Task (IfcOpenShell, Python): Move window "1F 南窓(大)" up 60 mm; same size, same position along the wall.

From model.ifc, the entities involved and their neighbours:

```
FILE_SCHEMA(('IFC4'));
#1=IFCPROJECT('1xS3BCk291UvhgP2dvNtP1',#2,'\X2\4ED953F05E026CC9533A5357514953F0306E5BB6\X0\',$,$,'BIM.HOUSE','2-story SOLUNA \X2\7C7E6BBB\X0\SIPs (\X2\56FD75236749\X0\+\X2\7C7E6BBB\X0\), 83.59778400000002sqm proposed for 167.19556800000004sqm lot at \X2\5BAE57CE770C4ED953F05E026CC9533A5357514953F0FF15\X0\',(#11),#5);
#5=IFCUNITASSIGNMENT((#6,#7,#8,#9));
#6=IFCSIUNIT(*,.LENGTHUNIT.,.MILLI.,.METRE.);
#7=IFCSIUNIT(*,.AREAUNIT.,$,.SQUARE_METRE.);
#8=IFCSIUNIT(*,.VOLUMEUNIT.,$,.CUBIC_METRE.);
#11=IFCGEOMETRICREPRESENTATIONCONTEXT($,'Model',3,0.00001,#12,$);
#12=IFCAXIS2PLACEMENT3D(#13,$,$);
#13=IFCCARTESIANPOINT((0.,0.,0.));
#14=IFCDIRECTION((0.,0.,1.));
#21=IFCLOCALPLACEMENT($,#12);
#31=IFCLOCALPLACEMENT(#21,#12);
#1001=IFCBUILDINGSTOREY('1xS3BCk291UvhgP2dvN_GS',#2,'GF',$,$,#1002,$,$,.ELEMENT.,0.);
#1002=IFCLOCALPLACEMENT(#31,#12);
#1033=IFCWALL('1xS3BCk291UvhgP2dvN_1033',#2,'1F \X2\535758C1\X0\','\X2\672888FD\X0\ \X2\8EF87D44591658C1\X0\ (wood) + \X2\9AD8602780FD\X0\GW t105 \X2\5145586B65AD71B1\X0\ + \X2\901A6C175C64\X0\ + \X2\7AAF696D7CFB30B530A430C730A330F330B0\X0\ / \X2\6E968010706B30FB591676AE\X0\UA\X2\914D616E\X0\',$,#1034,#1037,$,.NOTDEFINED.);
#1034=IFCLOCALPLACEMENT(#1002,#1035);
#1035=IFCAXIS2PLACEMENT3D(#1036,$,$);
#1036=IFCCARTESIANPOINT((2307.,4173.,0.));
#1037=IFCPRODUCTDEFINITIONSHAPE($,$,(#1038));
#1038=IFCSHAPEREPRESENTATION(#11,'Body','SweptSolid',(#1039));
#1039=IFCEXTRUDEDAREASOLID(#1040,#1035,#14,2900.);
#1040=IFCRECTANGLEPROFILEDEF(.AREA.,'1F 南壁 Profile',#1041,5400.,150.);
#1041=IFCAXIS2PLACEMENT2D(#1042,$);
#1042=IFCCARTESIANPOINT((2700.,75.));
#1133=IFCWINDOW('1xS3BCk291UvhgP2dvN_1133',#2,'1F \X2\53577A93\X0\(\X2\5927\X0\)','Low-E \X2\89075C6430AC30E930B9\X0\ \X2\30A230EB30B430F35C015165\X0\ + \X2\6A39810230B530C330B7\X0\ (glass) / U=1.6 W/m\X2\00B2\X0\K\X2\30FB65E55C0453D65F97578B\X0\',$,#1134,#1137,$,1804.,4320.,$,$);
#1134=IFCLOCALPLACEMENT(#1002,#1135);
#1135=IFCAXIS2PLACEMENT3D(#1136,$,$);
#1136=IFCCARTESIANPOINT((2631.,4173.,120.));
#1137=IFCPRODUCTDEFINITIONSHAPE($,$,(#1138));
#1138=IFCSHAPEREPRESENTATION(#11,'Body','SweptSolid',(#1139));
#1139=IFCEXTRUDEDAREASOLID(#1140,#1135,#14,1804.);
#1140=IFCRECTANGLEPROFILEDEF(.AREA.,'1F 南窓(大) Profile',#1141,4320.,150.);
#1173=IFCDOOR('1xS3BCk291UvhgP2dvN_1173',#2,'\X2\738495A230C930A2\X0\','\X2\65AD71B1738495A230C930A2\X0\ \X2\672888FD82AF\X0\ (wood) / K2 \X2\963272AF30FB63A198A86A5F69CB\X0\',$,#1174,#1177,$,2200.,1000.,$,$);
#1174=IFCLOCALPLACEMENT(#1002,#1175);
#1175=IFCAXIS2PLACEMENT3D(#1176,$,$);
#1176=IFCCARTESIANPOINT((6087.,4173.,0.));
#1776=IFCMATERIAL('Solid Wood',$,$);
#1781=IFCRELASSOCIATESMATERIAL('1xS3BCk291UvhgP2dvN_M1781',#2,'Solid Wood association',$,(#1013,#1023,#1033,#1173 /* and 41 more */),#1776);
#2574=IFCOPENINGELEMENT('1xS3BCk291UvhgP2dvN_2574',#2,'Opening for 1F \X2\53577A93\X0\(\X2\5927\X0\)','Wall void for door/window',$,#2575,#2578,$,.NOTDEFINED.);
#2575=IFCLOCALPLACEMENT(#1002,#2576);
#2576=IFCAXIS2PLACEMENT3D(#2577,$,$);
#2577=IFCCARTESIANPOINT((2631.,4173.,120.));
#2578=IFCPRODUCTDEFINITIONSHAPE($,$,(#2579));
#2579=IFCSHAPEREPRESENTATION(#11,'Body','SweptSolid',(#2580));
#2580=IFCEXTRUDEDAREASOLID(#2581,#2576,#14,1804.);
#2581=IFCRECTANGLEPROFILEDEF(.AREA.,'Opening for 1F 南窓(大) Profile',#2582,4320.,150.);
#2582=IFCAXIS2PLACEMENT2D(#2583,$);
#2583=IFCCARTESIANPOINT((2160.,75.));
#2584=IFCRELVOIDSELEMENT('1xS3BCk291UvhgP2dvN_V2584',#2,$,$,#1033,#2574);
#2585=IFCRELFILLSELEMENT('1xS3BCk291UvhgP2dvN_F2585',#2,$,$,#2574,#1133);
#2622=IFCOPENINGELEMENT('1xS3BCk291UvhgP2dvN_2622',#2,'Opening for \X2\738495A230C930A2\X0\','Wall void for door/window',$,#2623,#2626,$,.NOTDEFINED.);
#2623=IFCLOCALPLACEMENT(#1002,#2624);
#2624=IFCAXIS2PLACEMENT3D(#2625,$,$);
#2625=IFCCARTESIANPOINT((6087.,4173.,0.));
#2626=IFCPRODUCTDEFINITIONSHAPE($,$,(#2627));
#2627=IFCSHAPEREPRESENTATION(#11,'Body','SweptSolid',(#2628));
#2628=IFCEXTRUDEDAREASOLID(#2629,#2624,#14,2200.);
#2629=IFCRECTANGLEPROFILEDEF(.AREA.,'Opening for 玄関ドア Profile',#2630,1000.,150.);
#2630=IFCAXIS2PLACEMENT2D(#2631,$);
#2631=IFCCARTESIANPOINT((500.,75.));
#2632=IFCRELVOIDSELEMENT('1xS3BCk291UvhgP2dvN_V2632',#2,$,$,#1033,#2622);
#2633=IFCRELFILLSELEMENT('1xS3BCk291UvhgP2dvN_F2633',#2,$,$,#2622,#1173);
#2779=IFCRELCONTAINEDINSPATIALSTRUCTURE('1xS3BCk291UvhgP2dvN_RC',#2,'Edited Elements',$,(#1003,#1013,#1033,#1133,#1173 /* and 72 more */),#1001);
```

```python
import numpy as np
import ifcopenshell
import ifcopenshell.api.geometry
import ifcopenshell.util.placement
import ifcopenshell.util.unit

model = ifcopenshell.open("model.ifc")
unit_scale = ifcopenshell.util.unit.calculate_unit_scale(model)

window = model.by_id(1133)
opening = window.FillsVoids[0].RelatingOpeningElement
dz = 0.06 / unit_scale

shift = np.array([0.0, 0.0, dz])
# The window is not placed relative to its opening, so move both.
for product in (opening, window):
    matrix = ifcopenshell.util.placement.get_local_placement(product.ObjectPlacement)
    matrix[:3, 3] += shift
    ifcopenshell.api.geometry.edit_object_placement(model, product=product, matrix=matrix, is_si=False)

print(f"moved by {dz * unit_scale:+.3f} m")

model.write("model_rev.ifc")
```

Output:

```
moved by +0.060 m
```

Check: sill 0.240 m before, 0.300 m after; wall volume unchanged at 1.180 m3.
